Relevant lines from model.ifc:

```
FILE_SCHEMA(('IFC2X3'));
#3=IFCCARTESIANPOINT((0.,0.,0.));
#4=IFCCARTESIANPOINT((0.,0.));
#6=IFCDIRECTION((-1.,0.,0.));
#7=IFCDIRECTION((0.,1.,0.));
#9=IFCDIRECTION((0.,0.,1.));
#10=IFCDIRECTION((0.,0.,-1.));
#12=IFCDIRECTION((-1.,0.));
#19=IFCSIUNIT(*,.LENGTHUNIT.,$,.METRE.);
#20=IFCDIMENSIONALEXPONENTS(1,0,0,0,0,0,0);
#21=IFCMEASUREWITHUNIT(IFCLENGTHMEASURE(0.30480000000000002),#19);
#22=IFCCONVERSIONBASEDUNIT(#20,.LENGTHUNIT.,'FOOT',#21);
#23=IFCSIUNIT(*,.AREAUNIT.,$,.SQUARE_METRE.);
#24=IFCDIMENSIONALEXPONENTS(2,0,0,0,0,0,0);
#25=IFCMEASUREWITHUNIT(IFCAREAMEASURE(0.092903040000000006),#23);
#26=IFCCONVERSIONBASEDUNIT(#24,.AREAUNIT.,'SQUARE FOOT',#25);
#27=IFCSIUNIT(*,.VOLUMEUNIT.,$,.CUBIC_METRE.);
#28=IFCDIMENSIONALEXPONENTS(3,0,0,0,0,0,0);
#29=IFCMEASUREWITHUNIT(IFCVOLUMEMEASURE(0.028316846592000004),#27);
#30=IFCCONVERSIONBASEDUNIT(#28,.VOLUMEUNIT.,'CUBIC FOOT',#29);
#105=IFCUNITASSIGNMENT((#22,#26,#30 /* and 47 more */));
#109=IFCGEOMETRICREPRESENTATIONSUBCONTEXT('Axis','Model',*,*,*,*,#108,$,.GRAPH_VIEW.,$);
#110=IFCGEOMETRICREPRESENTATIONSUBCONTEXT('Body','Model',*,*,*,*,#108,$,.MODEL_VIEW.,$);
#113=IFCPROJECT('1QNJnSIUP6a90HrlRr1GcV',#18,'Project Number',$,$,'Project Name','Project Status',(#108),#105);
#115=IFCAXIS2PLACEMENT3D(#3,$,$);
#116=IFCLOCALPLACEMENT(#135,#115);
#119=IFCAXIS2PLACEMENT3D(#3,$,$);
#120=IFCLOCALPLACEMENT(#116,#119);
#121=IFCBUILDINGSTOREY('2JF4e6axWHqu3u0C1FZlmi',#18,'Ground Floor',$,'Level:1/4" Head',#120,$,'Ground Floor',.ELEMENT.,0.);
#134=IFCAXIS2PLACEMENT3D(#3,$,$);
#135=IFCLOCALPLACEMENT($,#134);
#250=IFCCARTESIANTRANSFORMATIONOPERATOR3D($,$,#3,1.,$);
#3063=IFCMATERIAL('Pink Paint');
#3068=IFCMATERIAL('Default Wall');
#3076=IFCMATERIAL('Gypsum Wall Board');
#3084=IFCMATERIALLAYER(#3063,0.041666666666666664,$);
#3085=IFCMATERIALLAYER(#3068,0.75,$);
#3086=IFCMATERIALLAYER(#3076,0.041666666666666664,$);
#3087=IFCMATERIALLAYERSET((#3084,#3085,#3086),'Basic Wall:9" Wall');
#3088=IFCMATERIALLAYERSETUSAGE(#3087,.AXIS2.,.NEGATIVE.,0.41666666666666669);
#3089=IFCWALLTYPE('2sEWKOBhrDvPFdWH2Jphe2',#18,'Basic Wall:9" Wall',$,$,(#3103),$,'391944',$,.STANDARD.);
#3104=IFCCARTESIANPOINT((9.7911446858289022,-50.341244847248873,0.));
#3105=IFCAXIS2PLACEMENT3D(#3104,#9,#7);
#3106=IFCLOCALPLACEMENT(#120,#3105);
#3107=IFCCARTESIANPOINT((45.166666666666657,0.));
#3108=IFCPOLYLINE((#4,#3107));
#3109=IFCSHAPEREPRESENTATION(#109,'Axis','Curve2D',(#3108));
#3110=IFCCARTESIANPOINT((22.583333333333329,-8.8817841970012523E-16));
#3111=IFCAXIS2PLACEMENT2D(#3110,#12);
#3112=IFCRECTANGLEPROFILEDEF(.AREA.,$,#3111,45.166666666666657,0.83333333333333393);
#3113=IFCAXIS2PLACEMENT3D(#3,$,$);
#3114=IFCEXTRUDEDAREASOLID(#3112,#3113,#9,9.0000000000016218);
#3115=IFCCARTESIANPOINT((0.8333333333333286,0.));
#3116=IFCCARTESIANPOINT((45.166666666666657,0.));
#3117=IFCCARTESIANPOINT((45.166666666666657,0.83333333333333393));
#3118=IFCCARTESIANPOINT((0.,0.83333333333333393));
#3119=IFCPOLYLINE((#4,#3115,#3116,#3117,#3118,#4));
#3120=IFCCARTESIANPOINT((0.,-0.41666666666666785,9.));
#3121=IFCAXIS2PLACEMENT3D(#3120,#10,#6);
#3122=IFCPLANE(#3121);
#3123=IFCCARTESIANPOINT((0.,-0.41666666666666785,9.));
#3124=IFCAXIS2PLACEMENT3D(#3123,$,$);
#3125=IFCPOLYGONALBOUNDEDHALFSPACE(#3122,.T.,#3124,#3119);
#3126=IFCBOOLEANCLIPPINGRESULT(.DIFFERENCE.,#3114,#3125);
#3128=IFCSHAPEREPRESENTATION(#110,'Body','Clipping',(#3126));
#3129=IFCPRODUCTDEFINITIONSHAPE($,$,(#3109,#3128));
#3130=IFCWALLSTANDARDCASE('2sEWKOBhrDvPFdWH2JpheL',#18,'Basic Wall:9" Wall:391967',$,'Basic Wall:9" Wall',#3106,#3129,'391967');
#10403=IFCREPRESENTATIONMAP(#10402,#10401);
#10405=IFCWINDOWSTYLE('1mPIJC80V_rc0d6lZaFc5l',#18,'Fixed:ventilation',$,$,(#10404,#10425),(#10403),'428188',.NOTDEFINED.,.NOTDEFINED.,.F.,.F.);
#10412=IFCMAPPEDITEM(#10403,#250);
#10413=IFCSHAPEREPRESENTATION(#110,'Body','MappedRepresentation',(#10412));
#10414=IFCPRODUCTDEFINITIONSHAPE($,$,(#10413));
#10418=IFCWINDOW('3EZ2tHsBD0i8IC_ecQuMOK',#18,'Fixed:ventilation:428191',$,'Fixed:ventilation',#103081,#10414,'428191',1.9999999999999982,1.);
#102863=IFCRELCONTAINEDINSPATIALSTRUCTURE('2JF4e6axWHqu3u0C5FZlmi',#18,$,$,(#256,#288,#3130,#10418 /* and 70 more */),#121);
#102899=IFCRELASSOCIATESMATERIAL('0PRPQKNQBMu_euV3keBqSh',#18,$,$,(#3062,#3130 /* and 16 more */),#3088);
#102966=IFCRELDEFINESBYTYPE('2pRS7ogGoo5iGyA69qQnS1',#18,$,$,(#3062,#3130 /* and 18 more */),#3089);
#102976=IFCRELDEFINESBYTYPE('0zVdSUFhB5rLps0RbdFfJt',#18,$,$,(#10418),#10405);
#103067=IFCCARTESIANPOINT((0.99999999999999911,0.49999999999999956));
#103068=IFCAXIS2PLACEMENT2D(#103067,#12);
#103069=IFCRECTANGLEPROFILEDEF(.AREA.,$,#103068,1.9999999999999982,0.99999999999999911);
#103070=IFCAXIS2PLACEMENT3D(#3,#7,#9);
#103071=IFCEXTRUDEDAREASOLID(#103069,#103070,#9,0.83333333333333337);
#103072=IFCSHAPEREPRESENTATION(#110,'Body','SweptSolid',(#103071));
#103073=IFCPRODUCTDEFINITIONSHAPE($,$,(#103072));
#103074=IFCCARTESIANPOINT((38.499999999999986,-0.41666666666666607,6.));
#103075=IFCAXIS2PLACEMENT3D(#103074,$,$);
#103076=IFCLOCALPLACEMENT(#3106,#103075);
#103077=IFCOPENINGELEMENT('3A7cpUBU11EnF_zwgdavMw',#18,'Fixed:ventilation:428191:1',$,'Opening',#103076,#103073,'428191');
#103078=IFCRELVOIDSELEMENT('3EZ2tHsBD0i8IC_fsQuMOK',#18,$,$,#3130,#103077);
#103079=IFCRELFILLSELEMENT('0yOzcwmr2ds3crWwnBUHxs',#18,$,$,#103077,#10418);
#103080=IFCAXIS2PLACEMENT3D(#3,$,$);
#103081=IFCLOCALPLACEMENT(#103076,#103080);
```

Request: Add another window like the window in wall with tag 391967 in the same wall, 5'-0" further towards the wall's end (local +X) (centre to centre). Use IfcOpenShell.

```python
import ifcopenshell
import ifcopenshell.api.feature
import ifcopenshell.api.geometry
import ifcopenshell.api.root
import ifcopenshell.geom
import ifcopenshell.util.element
import ifcopenshell.util.placement
import ifcopenshell.util.shape
import ifcopenshell.util.unit

model = ifcopenshell.open("model.ifc")
unit_scale = ifcopenshell.util.unit.calculate_unit_scale(model)
settings = ifcopenshell.geom.settings()


def volume(element):
    """Net volume in cubic metres, openings subtracted."""
    shape = ifcopenshell.geom.create_shape(settings, element)
    return ifcopenshell.util.shape.get_volume(shape.geometry)


def reuse_history(source, copy):
    """copy_class also copies each property set's owner history, people and application; keep the originals."""
    for rel in copy.IsDefinedBy:
        if rel.is_a("IfcRelDefinesByProperties") and (history := rel.RelatingPropertyDefinition.OwnerHistory):
            rel.RelatingPropertyDefinition.OwnerHistory = source.OwnerHistory
            ifcopenshell.util.element.remove_deep2(model, history)


window = model.by_guid("3EZ2tHsBD0i8IC_ecQuMOK")
opening = window.FillsVoids[0].RelatingOpeningElement
wall = opening.VoidsElements[0].RelatingBuildingElement
before = volume(wall)
shift = ifcopenshell.util.placement.get_local_placement(wall.ObjectPlacement)[:3, 0] * 60 * 0.0254 / unit_scale

# copy_class copies the void relationship, type, container and properties, but no geometry.
new_opening = ifcopenshell.api.root.copy_class(model, product=opening)
new_opening.Representation = ifcopenshell.util.element.copy_deep(
    model, opening.Representation, exclude=["IfcGeometricRepresentationContext", "IfcRepresentationMap"]
)
new_opening.Name = "Fixed:ventilation"
new_opening.Tag = None
new_window = ifcopenshell.api.root.copy_class(model, product=window)
new_window.Representation = ifcopenshell.util.element.copy_deep(
    model, window.Representation, exclude=["IfcGeometricRepresentationContext", "IfcRepresentationMap"]
)
new_window.Name = "Fixed:ventilation"
new_window.Tag = None
reuse_history(window, new_window)
fills = ifcopenshell.api.feature.add_filling(model, opening=new_opening, element=new_window)
fills.OwnerHistory = new_window.OwnerHistory  # required in IFC2X3

for old, new in ((opening, new_opening), (window, new_window)):
    matrix = ifcopenshell.util.placement.get_local_placement(old.ObjectPlacement)
    matrix[:3, 3] += shift
    ifcopenshell.api.geometry.edit_object_placement(model, product=new, matrix=matrix, is_si=False)

after = volume(wall)

print(f"wall volume {before:.3f} -> {after:.3f} m3")

model.write("model_updated.ifc")
```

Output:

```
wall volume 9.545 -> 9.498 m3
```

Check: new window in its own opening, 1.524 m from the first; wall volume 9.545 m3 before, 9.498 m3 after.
